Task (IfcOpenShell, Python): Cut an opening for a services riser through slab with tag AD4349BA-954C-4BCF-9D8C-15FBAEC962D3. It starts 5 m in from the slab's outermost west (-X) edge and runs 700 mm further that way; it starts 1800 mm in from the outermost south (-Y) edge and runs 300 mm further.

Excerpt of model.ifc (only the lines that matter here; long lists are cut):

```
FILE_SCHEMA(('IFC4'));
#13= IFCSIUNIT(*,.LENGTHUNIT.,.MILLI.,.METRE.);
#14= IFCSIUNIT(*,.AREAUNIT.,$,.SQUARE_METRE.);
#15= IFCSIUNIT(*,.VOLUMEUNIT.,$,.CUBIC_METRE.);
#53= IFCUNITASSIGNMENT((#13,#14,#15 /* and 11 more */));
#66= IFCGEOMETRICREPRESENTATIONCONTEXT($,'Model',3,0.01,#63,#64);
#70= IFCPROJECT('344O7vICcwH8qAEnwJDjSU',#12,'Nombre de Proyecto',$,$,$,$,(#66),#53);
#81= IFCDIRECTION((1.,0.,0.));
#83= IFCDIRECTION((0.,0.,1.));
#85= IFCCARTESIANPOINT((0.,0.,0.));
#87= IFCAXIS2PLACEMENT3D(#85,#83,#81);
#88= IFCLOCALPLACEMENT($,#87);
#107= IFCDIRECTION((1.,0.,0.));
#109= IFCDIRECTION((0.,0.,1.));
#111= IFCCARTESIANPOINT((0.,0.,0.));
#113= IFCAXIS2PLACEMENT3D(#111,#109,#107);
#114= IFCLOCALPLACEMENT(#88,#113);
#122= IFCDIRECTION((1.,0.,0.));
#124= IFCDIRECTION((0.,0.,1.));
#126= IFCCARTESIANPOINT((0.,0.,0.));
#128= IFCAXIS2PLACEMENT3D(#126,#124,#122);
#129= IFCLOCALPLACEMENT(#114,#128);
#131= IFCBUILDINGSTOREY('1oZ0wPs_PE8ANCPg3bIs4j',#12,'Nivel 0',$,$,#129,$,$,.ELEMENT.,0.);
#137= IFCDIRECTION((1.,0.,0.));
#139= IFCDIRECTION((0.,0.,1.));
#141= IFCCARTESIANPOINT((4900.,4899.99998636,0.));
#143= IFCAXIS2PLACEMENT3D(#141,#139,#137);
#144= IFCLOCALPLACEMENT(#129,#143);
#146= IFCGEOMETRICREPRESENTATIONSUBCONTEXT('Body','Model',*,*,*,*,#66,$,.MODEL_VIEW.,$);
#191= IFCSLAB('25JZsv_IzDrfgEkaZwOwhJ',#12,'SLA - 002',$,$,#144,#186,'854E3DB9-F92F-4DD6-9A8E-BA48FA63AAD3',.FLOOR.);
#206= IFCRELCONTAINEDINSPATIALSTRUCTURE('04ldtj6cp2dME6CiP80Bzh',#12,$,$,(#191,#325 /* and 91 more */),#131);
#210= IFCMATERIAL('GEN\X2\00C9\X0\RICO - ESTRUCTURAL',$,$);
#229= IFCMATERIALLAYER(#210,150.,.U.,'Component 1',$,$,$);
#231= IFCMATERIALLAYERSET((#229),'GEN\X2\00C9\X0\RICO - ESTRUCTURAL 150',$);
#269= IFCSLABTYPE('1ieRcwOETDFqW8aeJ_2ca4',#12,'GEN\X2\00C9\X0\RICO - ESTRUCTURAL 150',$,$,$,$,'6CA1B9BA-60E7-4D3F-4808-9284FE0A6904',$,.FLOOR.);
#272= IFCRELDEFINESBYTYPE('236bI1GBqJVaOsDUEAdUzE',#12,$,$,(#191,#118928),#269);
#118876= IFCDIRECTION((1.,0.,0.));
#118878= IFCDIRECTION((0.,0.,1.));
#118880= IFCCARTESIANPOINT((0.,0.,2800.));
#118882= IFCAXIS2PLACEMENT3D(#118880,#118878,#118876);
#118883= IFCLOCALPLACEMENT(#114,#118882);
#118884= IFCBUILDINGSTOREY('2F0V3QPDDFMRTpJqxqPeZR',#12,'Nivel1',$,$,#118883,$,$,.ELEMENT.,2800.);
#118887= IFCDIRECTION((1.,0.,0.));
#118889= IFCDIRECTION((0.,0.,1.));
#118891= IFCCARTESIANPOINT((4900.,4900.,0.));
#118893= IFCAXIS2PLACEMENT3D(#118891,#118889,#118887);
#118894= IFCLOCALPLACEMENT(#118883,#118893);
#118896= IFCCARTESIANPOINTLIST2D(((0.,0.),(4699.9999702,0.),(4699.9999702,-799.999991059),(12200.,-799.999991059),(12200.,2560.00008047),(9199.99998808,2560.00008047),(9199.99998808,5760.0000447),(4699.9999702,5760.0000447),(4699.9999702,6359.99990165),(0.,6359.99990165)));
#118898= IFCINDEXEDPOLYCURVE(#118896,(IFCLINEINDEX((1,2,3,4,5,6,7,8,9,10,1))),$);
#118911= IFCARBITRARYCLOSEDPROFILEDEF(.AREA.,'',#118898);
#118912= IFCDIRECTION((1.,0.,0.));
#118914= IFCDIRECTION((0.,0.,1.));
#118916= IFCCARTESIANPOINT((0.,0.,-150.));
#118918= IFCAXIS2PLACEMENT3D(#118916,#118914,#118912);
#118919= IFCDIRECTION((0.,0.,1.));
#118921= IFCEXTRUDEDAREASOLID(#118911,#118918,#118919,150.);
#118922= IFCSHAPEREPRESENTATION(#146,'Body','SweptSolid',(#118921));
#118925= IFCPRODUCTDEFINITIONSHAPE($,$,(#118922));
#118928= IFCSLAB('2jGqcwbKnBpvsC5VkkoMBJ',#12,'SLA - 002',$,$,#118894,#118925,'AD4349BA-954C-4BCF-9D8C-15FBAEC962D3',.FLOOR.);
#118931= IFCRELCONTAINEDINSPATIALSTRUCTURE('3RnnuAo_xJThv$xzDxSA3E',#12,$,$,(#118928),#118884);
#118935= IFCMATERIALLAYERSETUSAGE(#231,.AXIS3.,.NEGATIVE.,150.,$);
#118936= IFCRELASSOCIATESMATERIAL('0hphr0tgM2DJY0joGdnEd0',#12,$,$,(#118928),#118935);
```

```python
import numpy as np
import ifcopenshell
import ifcopenshell.api.feature
import ifcopenshell.api.geometry
import ifcopenshell.api.root
import ifcopenshell.geom
import ifcopenshell.util.placement
import ifcopenshell.util.representation
import ifcopenshell.util.shape
import ifcopenshell.util.unit

model = ifcopenshell.open("model.ifc")
unit_scale = ifcopenshell.util.unit.calculate_unit_scale(model)
settings = ifcopenshell.geom.settings()


def volume(element):
    """Net volume in cubic metres, openings subtracted."""
    shape = ifcopenshell.geom.create_shape(settings, element)
    return ifcopenshell.util.shape.get_volume(shape.geometry)


slab = model.by_id(118928)
before = volume(slab)

# Extent in the slab's own axes, in metres. The edges named are its -X and -Y sides.
slab_shape = ifcopenshell.geom.create_shape(settings, slab)
vertices = ifcopenshell.util.shape.get_vertices(slab_shape.geometry)
x_min, y_min, bottom = vertices.min(axis=0)
top = vertices[:, 2].max()

opening = ifcopenshell.api.root.create_entity(model, ifc_class="IfcOpeningElement", name="Services riser opening", predefined_type="OPENING")
context = ifcopenshell.util.representation.get_context(model, "Model", "Body", "MODEL_VIEW")
width, depth = 0.7, 0.3
outline = [(0.0, 0.0), (width, 0.0), (width, depth), (0.0, depth), (0.0, 0.0)]
# Overshoot both faces by 50 mm so the cut is clean.
shape = ifcopenshell.api.geometry.add_slab_representation(
    model, context=context, depth=top - bottom + 0.1, polyline=outline
)
ifcopenshell.api.geometry.assign_representation(model, product=opening, representation=shape)

matrix = ifcopenshell.util.placement.get_local_placement(slab.ObjectPlacement)
matrix[:, 3] = matrix @ np.append(np.array([x_min + 5, y_min + 1.8, bottom - 0.05]) / unit_scale, 1.0)
ifcopenshell.api.geometry.edit_object_placement(model, product=opening, matrix=matrix, is_si=False)
ifcopenshell.api.feature.add_feature(model, feature=opening, element=slab)

after = volume(slab)

print(f"slab volume {before:.3f} -> {after:.3f} m3")

model.write("model_v2.ifc")
```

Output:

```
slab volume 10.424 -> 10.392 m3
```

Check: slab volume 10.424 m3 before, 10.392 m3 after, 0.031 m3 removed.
